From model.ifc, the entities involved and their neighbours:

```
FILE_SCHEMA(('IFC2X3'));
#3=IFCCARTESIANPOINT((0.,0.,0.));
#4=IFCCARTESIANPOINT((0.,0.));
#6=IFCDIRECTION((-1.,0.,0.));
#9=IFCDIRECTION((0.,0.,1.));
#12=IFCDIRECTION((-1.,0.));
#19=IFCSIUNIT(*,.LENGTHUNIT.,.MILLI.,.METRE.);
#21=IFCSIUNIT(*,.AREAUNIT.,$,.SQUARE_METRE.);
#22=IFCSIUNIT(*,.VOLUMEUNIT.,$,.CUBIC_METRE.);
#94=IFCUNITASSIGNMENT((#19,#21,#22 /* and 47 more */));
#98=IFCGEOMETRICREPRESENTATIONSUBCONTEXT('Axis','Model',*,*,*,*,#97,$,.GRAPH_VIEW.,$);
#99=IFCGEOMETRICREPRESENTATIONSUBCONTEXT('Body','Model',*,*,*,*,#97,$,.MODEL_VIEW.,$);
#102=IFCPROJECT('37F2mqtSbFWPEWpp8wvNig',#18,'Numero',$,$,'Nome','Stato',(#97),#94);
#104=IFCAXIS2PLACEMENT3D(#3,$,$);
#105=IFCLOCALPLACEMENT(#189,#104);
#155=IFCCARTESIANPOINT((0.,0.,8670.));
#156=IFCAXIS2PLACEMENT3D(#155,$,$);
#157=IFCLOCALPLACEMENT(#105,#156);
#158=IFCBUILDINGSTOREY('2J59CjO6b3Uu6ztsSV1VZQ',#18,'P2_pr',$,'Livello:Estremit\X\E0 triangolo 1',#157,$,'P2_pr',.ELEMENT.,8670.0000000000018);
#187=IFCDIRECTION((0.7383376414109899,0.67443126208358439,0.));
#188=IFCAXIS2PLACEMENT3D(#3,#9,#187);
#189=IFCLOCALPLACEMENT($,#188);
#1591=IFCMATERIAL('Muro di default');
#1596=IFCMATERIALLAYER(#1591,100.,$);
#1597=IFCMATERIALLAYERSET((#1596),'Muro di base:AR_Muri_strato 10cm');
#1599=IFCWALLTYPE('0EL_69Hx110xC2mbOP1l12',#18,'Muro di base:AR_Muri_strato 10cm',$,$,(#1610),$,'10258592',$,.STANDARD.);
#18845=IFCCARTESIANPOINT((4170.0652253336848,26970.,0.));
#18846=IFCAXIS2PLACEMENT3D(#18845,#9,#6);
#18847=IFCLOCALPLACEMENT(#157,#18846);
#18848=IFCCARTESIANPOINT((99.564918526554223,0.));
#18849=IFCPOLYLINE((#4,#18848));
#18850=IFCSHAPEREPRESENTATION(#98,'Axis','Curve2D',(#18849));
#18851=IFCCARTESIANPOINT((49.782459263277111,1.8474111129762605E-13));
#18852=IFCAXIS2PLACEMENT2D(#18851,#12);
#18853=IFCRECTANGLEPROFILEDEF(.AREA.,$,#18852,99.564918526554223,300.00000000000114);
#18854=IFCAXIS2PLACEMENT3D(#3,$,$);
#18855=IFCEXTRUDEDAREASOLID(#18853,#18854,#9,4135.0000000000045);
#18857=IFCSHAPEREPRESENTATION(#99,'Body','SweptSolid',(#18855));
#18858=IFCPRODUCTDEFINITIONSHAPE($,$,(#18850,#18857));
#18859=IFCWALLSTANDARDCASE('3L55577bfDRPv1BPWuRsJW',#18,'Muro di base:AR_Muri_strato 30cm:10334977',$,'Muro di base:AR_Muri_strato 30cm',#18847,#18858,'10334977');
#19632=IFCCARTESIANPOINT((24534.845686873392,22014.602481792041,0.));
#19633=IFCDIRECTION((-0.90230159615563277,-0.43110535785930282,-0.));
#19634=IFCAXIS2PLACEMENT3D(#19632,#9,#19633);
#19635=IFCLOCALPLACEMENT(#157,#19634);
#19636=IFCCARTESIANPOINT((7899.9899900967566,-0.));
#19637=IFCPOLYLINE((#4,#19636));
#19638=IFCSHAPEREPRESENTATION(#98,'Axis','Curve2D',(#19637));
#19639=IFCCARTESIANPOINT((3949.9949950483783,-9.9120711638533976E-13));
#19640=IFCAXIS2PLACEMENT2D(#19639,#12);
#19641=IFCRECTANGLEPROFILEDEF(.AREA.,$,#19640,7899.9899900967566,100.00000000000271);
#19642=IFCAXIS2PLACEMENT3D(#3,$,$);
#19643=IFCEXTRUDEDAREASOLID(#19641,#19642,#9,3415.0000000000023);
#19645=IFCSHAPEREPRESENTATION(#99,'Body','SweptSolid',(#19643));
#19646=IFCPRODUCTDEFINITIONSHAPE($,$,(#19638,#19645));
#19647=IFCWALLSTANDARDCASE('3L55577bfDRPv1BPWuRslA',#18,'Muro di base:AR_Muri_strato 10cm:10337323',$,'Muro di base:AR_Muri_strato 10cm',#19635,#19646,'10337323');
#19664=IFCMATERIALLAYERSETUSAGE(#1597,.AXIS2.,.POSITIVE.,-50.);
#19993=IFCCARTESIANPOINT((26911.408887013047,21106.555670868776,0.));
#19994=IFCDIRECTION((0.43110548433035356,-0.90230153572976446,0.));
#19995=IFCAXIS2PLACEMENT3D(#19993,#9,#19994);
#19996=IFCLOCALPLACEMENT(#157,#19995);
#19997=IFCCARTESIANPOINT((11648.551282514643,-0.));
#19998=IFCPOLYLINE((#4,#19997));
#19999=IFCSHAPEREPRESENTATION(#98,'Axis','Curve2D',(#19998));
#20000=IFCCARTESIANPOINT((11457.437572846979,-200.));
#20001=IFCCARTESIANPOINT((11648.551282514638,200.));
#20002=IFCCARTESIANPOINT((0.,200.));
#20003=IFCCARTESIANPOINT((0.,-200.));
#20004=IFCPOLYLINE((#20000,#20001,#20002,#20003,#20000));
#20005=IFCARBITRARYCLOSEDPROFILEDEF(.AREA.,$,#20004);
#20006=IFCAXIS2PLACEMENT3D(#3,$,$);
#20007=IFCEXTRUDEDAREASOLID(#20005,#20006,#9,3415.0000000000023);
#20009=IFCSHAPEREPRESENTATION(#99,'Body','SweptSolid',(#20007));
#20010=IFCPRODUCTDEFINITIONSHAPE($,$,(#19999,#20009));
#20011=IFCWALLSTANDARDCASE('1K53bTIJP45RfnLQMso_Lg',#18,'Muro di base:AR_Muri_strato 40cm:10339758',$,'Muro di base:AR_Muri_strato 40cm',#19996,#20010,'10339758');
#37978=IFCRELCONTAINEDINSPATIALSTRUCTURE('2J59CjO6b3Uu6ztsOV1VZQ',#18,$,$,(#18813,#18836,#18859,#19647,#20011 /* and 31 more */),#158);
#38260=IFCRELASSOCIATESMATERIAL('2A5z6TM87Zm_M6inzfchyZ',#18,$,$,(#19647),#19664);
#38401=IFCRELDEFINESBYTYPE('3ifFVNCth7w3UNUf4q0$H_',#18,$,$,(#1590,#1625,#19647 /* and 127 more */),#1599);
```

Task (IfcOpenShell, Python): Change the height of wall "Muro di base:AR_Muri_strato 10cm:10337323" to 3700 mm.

```python
import ifcopenshell
import ifcopenshell.geom
import ifcopenshell.util.representation
import ifcopenshell.util.shape
import ifcopenshell.util.unit

model = ifcopenshell.open("model.ifc")
unit_scale = ifcopenshell.util.unit.calculate_unit_scale(model)
settings = ifcopenshell.geom.settings()


def volume(element):
    """Net volume in cubic metres, openings subtracted."""
    shape = ifcopenshell.geom.create_shape(settings, element)
    return ifcopenshell.util.shape.get_volume(shape.geometry)


wall = model.by_id(19647)
before = volume(wall)

body = ifcopenshell.util.representation.get_representation(wall, "Model", "Body")
solid = body.Items[0]
old_height = solid.Depth
solid.Depth = 3.7 / unit_scale
after = volume(wall)

print(f"height {old_height:g} -> {solid.Depth:g}, volume {before:.3f} -> {after:.3f} m3")

model.write("model_updated.ifc")
```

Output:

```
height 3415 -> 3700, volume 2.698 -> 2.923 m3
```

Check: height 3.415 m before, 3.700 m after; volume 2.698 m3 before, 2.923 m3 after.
